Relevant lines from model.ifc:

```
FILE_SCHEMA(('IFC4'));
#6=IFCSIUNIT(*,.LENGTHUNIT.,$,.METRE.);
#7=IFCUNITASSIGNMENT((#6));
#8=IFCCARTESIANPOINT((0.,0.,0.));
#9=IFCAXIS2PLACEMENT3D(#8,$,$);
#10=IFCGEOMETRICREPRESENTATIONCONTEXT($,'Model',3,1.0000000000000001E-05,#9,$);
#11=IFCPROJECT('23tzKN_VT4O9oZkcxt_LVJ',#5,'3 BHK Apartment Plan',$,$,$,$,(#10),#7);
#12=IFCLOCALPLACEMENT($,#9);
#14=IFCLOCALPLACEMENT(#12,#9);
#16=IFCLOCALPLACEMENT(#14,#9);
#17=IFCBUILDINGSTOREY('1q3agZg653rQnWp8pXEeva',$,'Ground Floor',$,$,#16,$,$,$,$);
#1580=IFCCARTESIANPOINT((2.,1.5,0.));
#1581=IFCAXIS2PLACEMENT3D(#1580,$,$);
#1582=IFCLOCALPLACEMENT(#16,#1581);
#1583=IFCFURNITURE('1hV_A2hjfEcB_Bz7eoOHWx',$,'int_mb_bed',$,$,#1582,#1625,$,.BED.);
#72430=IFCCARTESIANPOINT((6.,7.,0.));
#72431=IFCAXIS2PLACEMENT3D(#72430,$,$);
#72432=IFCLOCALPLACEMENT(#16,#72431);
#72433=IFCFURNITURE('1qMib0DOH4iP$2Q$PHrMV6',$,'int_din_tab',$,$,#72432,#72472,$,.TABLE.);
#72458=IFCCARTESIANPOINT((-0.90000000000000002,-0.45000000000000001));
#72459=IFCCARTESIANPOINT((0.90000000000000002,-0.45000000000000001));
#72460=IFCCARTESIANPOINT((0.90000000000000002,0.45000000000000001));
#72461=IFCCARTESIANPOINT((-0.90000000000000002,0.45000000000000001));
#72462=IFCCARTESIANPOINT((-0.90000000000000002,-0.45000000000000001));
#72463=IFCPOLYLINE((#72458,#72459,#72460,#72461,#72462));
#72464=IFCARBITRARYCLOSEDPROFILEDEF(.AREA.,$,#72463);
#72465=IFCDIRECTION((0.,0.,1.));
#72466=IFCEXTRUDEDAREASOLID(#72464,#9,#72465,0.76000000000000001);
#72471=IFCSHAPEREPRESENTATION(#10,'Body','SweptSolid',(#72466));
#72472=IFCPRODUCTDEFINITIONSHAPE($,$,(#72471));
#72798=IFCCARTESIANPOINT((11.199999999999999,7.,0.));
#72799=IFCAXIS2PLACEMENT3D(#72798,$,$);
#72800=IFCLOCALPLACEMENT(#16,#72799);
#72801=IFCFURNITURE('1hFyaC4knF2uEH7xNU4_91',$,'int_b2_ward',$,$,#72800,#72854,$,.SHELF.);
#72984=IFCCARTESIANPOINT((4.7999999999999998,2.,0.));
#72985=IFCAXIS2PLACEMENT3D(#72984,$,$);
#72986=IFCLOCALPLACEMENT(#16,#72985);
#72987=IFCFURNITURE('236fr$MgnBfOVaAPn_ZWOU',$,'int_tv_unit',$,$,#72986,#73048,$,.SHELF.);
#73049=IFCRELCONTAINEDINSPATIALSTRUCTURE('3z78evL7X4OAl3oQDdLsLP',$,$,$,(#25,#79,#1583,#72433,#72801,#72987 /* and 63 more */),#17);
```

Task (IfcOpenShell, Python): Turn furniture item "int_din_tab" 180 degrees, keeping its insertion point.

```python
import ifcopenshell
import ifcopenshell.api.geometry
import ifcopenshell.util.placement

model = ifcopenshell.open("model.ifc")

item = model.by_id(72433)
matrix = ifcopenshell.util.placement.get_local_placement(item.ObjectPlacement)
matrix = matrix @ ifcopenshell.util.placement.rotation(180, "Z")
ifcopenshell.api.geometry.edit_object_placement(model, product=item, matrix=matrix, is_si=False)

print(ifcopenshell.util.placement.get_local_placement(item.ObjectPlacement).round(3) + 0.0)

model.write("model_updated.ifc")
```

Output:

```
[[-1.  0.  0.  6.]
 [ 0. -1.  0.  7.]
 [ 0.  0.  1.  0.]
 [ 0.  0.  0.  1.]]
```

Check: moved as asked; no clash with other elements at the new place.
